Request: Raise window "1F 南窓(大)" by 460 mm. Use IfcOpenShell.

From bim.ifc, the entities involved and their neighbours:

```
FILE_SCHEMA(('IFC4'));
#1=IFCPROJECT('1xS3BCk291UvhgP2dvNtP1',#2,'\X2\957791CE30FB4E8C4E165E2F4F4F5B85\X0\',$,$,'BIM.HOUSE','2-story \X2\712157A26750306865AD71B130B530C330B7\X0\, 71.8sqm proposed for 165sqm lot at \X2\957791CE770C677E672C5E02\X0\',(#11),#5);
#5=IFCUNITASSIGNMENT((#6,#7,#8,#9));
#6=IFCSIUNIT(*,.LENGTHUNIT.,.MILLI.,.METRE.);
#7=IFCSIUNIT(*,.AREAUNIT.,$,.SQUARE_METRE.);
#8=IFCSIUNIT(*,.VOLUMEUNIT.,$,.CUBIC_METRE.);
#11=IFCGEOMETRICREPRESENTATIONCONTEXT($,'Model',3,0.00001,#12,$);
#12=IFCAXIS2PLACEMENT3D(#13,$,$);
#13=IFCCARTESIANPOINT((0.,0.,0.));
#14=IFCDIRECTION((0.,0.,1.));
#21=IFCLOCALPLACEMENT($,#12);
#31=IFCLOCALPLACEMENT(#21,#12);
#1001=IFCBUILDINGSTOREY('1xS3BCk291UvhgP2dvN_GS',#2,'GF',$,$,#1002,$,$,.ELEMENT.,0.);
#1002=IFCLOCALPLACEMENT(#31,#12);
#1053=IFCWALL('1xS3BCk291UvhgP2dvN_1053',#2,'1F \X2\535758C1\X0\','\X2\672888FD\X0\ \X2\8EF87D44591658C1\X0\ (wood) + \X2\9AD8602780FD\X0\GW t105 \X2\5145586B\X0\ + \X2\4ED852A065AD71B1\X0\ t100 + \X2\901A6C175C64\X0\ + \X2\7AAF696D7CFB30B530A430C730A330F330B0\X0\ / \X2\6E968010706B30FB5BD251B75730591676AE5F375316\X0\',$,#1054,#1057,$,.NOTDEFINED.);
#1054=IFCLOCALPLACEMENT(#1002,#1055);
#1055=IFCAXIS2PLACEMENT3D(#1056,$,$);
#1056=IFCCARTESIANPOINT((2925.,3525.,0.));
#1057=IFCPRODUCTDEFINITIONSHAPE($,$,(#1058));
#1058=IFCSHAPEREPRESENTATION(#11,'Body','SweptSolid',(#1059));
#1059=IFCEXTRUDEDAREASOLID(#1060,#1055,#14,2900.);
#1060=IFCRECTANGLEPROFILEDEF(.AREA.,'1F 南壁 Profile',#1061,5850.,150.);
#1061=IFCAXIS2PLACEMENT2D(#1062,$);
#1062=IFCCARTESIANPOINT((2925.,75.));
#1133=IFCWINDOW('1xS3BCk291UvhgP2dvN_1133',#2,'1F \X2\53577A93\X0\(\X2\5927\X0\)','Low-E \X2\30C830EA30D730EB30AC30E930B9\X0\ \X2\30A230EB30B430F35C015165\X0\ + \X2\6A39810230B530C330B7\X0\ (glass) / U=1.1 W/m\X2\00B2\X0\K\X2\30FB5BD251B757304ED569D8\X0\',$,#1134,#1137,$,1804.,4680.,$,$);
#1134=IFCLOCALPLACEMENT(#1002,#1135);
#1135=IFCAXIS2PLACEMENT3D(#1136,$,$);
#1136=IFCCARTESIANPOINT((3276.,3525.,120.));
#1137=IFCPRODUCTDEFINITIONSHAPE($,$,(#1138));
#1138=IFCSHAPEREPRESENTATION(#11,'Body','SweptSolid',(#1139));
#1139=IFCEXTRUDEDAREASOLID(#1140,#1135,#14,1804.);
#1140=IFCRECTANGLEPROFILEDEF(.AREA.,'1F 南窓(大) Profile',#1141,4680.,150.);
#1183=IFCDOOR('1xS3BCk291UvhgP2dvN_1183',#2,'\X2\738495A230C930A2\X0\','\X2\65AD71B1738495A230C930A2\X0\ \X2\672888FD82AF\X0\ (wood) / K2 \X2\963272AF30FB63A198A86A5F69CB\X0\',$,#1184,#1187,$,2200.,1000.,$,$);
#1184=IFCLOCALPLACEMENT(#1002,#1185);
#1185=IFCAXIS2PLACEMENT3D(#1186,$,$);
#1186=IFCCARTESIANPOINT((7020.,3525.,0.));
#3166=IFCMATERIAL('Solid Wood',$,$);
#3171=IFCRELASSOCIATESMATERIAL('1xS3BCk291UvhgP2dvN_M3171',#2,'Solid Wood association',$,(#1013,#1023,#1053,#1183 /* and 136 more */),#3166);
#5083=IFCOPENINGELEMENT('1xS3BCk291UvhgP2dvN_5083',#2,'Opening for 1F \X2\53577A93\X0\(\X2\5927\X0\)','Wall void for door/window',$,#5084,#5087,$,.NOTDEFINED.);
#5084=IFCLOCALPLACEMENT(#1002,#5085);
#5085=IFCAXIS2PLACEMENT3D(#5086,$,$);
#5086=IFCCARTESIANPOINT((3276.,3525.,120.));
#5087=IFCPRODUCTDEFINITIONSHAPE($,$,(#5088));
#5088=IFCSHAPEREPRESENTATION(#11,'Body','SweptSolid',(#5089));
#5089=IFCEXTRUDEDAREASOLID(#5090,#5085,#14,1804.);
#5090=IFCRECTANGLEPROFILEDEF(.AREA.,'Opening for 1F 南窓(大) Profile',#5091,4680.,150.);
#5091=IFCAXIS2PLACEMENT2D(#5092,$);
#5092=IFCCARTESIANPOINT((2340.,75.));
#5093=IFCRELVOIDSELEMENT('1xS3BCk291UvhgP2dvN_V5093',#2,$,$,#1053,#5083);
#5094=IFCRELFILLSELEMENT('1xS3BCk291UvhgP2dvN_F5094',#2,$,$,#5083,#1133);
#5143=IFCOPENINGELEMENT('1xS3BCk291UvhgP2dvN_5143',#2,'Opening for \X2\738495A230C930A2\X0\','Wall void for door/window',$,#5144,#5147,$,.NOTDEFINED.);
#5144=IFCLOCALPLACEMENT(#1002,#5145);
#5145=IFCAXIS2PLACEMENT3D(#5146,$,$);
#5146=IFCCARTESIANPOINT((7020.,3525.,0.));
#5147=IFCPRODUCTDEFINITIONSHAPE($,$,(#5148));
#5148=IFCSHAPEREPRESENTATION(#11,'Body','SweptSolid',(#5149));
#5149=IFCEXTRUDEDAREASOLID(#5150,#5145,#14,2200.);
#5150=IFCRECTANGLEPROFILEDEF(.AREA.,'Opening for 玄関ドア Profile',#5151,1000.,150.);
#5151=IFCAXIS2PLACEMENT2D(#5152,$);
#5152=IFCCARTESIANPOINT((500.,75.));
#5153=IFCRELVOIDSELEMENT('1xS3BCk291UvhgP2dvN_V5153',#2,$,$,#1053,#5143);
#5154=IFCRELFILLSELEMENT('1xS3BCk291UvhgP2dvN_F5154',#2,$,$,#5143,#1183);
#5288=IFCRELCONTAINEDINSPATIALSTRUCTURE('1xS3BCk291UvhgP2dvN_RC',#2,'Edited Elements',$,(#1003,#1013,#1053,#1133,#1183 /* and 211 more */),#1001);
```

```python
import numpy as np
import ifcopenshell
import ifcopenshell.api.geometry
import ifcopenshell.util.placement
import ifcopenshell.util.unit

model = ifcopenshell.open("bim.ifc")
unit_scale = ifcopenshell.util.unit.calculate_unit_scale(model)

window = model.by_guid("1xS3BCk291UvhgP2dvN_1133")
opening = window.FillsVoids[0].RelatingOpeningElement
dz = 0.46 / unit_scale

shift = np.array([0.0, 0.0, dz])
# The window is not placed relative to its opening, so move both.
for product in (opening, window):
    matrix = ifcopenshell.util.placement.get_local_placement(product.ObjectPlacement)
    matrix[:3, 3] += shift
    ifcopenshell.api.geometry.edit_object_placement(model, product=product, matrix=matrix, is_si=False)

print(f"moved by {dz * unit_scale:+.3f} m")

model.write("bim-out.ifc")
```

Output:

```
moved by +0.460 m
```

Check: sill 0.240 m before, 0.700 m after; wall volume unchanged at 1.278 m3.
